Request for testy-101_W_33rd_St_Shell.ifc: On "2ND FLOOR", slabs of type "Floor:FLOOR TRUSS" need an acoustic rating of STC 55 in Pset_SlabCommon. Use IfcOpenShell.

First a look at what the model holds.

```python
import ifcopenshell
import ifcopenshell.util.element

model = ifcopenshell.open("testy-101_W_33rd_St_Shell.ifc")
print(model.schema)
storey = next(s for s in model.by_type("IfcBuildingStorey") if s.Name == "2ND FLOOR")
slabs = [e for e in ifcopenshell.util.element.get_decomposition(storey) if e.is_a("IfcSlab")]
seen = {}
for e in slabs:
    element_type = ifcopenshell.util.element.get_type(e)
    key = (element_type.Name if element_type != e and element_type else None, ifcopenshell.util.element.get_pset(e, "Pset_SlabCommon", "AcousticRating"))
    seen[key] = seen.get(key, 0) + 1
for (name, value), count in sorted(seen.items(), key=str):
    print(count, "x", name, "|", value)
```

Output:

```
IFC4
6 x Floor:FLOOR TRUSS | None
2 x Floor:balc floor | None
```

```python
import ifcopenshell
import ifcopenshell.api.pset
import ifcopenshell.util.element

model = ifcopenshell.open("testy-101_W_33rd_St_Shell.ifc")

storey = next(s for s in model.by_type("IfcBuildingStorey") if s.Name == "2ND FLOOR")
slabs = [e for e in ifcopenshell.util.element.get_decomposition(storey) if e.is_a("IfcSlab")]

count = 0
for e in slabs:
    element_type = ifcopenshell.util.element.get_type(e)
    if element_type in (None, e) or element_type.Name != "Floor:FLOOR TRUSS":
        continue
    # add_pset returns the element's existing set when there is one.
    pset = ifcopenshell.api.pset.add_pset(model, product=e, name="Pset_SlabCommon")
    ifcopenshell.api.pset.edit_pset(model, pset=pset, properties={"AcousticRating": "STC 55"})
    count += 1

print(count, "slabs updated")

model.write("testy-101_W_33rd_St_Shell-out.ifc")
```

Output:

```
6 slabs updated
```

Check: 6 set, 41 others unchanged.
